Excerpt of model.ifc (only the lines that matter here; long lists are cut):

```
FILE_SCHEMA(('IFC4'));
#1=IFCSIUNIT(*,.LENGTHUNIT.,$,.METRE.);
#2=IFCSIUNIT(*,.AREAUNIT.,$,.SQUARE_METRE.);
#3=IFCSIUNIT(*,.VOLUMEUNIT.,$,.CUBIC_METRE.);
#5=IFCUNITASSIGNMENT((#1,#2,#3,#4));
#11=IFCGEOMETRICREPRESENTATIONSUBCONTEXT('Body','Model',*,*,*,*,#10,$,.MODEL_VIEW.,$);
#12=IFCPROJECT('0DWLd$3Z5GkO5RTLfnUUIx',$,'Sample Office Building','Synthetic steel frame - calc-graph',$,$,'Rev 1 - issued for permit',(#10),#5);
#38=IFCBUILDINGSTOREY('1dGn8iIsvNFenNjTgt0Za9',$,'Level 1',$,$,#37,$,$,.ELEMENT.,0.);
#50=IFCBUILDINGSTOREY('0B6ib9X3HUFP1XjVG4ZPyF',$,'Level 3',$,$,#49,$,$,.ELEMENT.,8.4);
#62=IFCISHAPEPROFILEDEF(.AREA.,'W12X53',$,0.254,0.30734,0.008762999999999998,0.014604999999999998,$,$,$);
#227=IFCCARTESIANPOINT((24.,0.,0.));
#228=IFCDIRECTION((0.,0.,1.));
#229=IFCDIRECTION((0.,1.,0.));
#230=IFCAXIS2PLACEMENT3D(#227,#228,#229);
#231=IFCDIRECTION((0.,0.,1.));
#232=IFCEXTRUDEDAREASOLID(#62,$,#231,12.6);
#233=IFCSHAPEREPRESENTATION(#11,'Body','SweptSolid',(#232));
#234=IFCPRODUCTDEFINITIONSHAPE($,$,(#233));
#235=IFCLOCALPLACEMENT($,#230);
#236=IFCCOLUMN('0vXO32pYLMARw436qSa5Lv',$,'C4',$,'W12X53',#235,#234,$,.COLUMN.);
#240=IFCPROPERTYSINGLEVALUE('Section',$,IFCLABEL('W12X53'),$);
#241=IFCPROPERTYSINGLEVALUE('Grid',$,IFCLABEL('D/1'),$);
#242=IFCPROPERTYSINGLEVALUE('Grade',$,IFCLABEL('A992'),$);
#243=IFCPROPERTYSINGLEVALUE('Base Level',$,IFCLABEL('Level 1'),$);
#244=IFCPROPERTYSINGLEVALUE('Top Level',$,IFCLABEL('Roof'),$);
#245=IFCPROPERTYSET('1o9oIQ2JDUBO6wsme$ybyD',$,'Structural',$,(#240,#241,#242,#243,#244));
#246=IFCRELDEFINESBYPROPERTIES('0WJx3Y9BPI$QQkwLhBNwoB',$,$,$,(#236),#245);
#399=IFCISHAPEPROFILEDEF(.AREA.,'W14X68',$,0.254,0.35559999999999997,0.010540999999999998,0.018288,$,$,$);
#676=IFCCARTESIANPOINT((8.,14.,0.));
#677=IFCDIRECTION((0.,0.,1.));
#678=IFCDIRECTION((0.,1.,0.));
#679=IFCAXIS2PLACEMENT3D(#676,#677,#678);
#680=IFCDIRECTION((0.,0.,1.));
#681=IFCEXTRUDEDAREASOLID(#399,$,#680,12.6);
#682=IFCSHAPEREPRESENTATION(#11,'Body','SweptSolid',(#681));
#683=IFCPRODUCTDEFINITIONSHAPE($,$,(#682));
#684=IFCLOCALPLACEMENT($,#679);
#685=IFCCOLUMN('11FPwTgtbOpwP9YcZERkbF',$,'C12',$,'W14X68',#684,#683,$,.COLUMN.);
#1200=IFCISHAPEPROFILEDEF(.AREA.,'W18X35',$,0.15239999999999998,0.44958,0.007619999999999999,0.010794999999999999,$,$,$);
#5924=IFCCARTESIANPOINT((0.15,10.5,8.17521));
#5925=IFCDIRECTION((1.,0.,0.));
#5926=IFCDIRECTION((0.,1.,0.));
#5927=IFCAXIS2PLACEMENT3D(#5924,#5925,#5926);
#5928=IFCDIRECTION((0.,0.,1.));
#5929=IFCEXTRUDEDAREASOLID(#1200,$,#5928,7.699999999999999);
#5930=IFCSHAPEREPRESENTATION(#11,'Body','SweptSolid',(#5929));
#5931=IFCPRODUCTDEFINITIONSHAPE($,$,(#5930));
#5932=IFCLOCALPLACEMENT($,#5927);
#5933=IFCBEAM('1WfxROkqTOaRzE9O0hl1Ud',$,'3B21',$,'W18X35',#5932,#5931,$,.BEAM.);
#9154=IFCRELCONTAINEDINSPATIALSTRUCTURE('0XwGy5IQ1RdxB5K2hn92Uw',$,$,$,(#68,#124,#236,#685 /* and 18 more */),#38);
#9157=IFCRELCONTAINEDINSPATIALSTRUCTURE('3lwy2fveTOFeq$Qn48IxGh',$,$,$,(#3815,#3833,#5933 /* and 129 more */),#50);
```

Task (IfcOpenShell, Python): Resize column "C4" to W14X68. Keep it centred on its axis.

```python
import ifcopenshell
import ifcopenshell.api.pset
import ifcopenshell.util.element
import ifcopenshell.util.representation

model = ifcopenshell.open("model.ifc")

member = model.by_id(236)
source = next(p for p in model.by_type("IfcIShapeProfileDef") if p.ProfileName == "W14X68")

body = ifcopenshell.util.representation.get_representation(member, "Model", "Body")
solid = body.Items[0]
old_profile = solid.SweptArea

# Copy the section's sizes but keep this member's own profile position.
profile = ifcopenshell.util.element.copy(model, source)
profile.Position = old_profile.Position
solid.SweptArea = profile
if not model.get_total_inverses(old_profile):
    ifcopenshell.util.element.remove_deep2(model, old_profile)
member.ObjectType = member.ObjectType.replace("W12X53", "W14X68")
pset = model.by_id(ifcopenshell.util.element.get_pset(member, "Structural", should_inherit=False)["id"])
ifcopenshell.api.pset.edit_pset(model, pset=pset, properties={"Section": "W14X68"})

print(solid.SweptArea)

model.write("model-out.ifc")
```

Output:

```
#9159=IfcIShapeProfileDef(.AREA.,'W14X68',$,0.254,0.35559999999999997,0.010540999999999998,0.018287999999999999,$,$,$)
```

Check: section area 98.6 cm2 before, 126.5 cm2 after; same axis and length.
